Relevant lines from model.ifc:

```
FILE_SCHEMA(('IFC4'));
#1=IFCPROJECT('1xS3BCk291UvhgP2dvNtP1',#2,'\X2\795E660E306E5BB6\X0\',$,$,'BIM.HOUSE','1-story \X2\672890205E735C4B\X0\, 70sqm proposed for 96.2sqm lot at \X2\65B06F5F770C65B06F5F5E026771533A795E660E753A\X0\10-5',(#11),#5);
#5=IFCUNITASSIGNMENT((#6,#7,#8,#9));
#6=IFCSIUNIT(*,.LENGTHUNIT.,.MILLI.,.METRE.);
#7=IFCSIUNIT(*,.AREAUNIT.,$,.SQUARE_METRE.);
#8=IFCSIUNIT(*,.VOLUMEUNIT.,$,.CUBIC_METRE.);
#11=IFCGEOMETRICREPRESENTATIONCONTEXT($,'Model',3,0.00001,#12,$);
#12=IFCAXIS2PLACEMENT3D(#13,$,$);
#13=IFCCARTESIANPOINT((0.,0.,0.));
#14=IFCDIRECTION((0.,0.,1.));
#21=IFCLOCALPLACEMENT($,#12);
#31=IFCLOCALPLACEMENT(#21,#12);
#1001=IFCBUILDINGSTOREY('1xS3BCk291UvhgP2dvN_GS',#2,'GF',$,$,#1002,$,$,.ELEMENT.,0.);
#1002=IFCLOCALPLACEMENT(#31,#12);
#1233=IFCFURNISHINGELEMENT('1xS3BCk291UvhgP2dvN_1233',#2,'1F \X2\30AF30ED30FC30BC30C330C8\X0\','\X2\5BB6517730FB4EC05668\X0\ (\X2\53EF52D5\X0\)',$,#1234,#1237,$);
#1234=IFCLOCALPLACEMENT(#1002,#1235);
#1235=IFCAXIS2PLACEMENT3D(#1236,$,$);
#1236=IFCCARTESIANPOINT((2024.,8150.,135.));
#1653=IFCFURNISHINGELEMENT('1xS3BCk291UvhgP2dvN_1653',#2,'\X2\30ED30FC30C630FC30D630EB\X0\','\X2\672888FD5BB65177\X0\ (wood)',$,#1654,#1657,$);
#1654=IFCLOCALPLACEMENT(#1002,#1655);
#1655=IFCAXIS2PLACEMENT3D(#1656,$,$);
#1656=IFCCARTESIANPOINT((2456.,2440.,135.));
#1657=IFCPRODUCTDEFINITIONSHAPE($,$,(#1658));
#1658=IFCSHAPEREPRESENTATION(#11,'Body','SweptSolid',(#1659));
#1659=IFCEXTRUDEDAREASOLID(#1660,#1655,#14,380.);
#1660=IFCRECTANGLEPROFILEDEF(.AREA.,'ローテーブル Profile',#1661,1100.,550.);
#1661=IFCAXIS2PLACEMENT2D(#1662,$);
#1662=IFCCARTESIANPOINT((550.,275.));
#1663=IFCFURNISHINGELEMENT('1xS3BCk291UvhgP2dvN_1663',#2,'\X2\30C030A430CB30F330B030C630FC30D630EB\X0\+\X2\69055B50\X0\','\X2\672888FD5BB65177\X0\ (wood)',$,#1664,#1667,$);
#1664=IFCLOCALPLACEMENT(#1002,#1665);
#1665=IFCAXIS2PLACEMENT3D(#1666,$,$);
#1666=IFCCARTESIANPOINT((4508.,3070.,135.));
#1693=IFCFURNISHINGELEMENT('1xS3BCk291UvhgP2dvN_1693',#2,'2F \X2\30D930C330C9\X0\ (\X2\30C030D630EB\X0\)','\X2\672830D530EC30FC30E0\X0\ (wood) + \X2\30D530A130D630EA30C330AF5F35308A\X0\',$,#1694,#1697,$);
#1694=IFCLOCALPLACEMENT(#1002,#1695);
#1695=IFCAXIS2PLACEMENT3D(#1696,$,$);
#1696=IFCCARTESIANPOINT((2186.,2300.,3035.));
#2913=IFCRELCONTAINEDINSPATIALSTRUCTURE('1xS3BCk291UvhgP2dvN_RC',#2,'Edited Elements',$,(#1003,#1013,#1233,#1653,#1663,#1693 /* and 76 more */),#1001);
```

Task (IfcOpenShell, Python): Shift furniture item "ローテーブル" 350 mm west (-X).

```python
import ifcopenshell
import ifcopenshell.api.geometry
import ifcopenshell.util.placement

model = ifcopenshell.open("model.ifc")

item = model.by_id(1653)
matrix = ifcopenshell.util.placement.get_local_placement(item.ObjectPlacement)
matrix[0, 3] -= 350.0
ifcopenshell.api.geometry.edit_object_placement(model, product=item, matrix=matrix, is_si=False)

print(ifcopenshell.util.placement.get_local_placement(item.ObjectPlacement).round(3) + 0.0)

model.write("model_rev.ifc")
```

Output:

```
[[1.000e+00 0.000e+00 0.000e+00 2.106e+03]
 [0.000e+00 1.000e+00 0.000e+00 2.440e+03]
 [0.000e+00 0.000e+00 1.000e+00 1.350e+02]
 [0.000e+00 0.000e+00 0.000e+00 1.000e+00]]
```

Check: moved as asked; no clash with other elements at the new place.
